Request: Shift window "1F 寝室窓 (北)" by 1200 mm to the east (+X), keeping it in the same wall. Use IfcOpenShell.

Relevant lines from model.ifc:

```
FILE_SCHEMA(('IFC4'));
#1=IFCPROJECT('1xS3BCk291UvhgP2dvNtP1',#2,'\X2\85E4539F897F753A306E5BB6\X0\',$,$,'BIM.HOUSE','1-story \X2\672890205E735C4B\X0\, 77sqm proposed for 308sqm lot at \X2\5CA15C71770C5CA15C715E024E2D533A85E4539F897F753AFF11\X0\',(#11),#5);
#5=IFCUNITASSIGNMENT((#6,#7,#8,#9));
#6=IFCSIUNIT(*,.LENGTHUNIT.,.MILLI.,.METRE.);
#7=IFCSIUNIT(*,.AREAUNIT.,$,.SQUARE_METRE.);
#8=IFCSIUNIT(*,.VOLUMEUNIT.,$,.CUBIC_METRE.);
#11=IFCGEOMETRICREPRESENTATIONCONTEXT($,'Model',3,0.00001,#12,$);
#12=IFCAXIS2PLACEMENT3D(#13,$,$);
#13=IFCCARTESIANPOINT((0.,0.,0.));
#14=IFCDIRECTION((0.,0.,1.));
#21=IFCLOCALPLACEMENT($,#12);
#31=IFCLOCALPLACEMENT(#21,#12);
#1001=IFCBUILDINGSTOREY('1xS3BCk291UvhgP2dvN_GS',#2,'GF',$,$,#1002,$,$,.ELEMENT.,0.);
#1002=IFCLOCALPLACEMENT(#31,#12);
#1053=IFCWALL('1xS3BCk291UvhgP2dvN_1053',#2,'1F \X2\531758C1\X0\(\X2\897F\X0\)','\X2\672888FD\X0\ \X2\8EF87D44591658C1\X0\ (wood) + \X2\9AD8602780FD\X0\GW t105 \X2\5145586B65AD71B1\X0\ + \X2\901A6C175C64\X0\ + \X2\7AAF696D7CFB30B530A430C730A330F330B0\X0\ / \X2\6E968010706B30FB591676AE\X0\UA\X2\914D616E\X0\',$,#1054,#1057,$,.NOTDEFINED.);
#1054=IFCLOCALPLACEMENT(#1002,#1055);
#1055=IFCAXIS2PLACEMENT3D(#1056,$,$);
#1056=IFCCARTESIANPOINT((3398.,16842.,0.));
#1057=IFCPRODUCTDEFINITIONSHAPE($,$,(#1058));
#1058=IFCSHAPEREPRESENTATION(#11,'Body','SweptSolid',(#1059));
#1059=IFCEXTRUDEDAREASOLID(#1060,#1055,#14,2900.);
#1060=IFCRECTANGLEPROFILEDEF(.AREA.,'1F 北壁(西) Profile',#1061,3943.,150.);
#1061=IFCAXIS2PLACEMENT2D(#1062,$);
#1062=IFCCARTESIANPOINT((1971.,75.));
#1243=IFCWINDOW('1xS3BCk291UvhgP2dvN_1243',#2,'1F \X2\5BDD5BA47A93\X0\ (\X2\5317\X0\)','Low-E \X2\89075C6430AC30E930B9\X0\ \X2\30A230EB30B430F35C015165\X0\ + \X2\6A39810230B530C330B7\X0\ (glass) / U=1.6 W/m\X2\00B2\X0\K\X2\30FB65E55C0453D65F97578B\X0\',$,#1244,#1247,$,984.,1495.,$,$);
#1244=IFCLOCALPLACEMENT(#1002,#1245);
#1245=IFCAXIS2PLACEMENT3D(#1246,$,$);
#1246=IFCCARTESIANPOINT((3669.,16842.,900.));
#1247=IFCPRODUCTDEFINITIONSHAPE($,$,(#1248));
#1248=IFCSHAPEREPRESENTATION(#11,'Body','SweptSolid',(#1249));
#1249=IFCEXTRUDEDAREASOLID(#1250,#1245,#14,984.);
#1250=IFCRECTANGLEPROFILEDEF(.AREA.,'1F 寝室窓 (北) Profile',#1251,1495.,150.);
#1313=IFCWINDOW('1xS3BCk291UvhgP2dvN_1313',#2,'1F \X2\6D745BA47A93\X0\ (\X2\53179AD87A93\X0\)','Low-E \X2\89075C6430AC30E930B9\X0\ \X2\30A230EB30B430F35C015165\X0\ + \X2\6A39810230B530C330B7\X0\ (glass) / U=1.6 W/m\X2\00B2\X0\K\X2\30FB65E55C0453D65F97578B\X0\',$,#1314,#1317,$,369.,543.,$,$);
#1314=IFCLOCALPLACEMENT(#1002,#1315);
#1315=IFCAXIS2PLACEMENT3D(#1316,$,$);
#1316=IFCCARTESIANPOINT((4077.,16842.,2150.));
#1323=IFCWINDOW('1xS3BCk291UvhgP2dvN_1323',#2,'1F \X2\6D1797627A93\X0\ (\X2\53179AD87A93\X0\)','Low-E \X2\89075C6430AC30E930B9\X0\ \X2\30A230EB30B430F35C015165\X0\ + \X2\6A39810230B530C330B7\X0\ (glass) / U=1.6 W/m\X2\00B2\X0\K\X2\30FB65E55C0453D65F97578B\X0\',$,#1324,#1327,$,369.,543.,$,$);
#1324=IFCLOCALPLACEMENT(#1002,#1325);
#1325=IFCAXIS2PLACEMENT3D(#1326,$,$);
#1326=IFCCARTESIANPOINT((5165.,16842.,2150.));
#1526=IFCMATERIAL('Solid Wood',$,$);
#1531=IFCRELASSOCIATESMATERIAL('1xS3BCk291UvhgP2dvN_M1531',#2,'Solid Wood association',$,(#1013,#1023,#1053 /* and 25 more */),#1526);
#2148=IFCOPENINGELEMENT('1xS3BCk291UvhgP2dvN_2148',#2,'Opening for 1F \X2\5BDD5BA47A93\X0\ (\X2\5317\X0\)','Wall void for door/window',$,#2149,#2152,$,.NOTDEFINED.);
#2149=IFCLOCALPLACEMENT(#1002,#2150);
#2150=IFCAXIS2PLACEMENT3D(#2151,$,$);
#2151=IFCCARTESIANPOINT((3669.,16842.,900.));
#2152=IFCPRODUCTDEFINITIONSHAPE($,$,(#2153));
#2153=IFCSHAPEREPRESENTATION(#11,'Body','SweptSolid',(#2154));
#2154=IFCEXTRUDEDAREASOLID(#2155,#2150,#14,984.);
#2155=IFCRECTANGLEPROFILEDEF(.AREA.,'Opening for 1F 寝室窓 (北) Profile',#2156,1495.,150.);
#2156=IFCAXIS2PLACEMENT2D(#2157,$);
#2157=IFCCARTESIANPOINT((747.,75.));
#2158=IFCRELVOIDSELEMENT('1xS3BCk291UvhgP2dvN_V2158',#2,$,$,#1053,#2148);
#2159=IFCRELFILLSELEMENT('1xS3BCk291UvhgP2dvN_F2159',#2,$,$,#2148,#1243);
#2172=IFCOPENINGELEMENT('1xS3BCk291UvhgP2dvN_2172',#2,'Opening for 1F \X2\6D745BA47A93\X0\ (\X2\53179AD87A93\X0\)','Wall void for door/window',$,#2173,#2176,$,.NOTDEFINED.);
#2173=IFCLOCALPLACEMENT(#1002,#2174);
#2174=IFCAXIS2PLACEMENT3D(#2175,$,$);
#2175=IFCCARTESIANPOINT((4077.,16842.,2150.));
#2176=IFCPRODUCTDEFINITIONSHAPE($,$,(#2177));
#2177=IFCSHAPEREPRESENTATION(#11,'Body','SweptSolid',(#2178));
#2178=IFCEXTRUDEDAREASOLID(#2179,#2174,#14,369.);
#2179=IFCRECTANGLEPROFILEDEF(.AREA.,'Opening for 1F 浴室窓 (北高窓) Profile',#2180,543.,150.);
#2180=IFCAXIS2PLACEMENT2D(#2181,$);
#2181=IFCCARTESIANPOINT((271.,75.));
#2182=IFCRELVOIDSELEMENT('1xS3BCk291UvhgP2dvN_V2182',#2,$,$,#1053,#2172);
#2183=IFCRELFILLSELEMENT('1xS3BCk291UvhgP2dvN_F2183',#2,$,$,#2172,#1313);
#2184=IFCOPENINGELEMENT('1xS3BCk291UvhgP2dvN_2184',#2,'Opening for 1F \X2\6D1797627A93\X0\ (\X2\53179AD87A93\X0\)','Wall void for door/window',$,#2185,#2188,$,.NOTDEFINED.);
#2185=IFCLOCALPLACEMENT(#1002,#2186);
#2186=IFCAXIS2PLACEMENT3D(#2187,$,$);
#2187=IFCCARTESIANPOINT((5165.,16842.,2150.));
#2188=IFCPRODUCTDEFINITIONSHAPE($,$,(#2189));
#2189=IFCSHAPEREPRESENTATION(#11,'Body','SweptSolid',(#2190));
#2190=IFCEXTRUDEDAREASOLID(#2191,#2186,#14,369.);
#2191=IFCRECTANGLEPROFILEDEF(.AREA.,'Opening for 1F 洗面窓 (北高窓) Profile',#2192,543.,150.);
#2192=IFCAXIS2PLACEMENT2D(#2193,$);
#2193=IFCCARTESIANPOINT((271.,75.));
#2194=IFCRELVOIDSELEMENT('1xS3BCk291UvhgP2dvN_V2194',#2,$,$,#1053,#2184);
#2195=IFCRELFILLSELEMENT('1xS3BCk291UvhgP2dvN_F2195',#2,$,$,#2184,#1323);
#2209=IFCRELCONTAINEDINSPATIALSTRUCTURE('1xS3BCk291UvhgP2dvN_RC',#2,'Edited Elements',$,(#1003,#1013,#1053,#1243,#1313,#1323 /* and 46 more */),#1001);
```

```python
import ifcopenshell
import ifcopenshell.api.geometry
import ifcopenshell.util.placement
import ifcopenshell.util.unit

model = ifcopenshell.open("model.ifc")
unit_scale = ifcopenshell.util.unit.calculate_unit_scale(model)

window = model.by_guid("1xS3BCk291UvhgP2dvN_1243")
opening = window.FillsVoids[0].RelatingOpeningElement
wall = opening.VoidsElements[0].RelatingBuildingElement

wall_matrix = ifcopenshell.util.placement.get_local_placement(wall.ObjectPlacement)
shift = wall_matrix[:3, 0] * 1.2 / unit_scale
before = ifcopenshell.util.placement.get_local_placement(window.ObjectPlacement)[:3, 3].copy()

# The window is not placed relative to its opening, so move both.
for product in (opening, window):
    matrix = ifcopenshell.util.placement.get_local_placement(product.ObjectPlacement)
    matrix[:3, 3] += shift
    ifcopenshell.api.geometry.edit_object_placement(model, product=product, matrix=matrix, is_si=False)

after = ifcopenshell.util.placement.get_local_placement(window.ObjectPlacement)[:3, 3]
print("window moved by", (after - before).round(3) + 0.0)

model.write("model-out.ifc")
```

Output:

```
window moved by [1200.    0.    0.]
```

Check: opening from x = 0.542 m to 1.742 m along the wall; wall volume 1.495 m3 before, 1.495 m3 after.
